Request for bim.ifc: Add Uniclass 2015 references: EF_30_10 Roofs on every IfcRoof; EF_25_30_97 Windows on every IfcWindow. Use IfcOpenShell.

First a look at what the model holds.

```python
import ifcopenshell

model = ifcopenshell.open("bim.ifc")
print(model.schema)
print("classifications:", [c.Name for c in model.by_type("IfcClassification")])
for ifc_class in ("IfcDoor", "IfcRoof", "IfcStair", "IfcWall", "IfcWindow"):
    print(ifc_class, len(model.by_type(ifc_class)))
```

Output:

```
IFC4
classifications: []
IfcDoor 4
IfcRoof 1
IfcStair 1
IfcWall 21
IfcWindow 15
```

```python
import ifcopenshell
import ifcopenshell.api.classification

model = ifcopenshell.open("bim.ifc")

system = ifcopenshell.api.classification.add_classification(model, classification="Uniclass 2015")

codes = {
    "IfcRoof": ("EF_30_10", "Roofs"),
    "IfcWindow": ("EF_25_30_97", "Windows"),
}
for ifc_class, (code, name) in codes.items():
    products = model.by_type(ifc_class)
    ifcopenshell.api.classification.add_reference(
        model, products=products, classification=system, identification=code, name=name
    )
    print(code, len(products))

model.write("bim-out.ifc")
```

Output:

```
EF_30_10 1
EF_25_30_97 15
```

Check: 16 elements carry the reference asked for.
